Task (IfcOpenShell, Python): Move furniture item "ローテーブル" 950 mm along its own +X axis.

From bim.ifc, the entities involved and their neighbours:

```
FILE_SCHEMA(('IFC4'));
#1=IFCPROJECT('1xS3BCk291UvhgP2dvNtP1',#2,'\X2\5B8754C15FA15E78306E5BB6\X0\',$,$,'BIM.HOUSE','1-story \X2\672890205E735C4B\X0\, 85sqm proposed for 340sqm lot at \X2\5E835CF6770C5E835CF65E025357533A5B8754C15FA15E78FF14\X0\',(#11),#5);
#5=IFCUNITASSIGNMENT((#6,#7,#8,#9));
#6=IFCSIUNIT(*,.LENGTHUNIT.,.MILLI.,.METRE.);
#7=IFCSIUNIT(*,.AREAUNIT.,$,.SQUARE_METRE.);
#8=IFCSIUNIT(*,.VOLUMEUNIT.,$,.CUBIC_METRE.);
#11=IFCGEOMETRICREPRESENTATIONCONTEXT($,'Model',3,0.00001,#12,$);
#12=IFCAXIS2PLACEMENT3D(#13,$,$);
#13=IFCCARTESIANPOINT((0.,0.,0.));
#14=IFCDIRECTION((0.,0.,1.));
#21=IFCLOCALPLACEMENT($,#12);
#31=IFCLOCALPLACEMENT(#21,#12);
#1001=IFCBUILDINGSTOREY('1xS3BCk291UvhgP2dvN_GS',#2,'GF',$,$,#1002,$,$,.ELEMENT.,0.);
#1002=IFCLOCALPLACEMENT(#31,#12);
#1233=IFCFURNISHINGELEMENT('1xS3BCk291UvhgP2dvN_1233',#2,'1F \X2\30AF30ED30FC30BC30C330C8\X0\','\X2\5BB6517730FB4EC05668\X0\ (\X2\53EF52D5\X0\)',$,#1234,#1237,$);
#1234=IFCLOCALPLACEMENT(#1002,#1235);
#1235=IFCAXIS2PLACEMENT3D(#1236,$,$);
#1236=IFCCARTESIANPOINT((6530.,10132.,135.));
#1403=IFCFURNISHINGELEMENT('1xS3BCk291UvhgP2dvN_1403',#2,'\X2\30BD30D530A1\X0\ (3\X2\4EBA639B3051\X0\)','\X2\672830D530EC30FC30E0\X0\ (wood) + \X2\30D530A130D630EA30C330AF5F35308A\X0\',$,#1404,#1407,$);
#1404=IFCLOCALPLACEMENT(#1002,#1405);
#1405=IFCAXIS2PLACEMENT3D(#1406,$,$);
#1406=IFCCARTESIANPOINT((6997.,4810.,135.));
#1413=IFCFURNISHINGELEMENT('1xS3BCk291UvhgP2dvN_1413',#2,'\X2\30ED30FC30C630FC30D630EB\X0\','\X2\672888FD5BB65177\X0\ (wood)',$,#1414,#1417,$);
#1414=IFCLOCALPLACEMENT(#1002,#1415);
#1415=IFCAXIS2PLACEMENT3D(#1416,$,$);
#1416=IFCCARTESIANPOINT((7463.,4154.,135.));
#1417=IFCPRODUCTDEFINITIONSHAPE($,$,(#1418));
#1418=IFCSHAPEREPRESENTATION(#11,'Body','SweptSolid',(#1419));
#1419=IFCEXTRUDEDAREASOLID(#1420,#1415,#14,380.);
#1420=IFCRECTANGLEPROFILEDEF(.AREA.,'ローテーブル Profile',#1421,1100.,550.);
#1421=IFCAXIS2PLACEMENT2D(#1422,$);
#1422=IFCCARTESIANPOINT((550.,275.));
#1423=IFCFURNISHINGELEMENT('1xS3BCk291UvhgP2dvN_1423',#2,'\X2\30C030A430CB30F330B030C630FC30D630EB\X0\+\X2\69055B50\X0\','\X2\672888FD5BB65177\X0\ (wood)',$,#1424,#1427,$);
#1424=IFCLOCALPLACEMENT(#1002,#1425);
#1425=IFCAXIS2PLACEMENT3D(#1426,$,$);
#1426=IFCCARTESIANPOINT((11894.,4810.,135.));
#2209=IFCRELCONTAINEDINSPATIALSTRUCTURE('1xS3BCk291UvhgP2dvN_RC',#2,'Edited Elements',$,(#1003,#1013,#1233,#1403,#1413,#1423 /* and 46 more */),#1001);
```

```python
import ifcopenshell
import ifcopenshell.api.geometry
import ifcopenshell.util.placement
import ifcopenshell.util.unit

model = ifcopenshell.open("bim.ifc")
unit_scale = ifcopenshell.util.unit.calculate_unit_scale(model)

item = model.by_guid("1xS3BCk291UvhgP2dvN_1413")
matrix = ifcopenshell.util.placement.get_local_placement(item.ObjectPlacement)
matrix[:3, 3] += matrix[:3, 0] * 0.95 / unit_scale
ifcopenshell.api.geometry.edit_object_placement(model, product=item, matrix=matrix, is_si=False)

print(ifcopenshell.util.placement.get_local_placement(item.ObjectPlacement).round(3) + 0.0)

model.write("bim_rev.ifc")
```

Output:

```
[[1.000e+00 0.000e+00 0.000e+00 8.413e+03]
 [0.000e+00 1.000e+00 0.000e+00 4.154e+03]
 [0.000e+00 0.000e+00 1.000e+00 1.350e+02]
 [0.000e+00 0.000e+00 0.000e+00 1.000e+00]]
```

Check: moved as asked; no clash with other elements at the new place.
